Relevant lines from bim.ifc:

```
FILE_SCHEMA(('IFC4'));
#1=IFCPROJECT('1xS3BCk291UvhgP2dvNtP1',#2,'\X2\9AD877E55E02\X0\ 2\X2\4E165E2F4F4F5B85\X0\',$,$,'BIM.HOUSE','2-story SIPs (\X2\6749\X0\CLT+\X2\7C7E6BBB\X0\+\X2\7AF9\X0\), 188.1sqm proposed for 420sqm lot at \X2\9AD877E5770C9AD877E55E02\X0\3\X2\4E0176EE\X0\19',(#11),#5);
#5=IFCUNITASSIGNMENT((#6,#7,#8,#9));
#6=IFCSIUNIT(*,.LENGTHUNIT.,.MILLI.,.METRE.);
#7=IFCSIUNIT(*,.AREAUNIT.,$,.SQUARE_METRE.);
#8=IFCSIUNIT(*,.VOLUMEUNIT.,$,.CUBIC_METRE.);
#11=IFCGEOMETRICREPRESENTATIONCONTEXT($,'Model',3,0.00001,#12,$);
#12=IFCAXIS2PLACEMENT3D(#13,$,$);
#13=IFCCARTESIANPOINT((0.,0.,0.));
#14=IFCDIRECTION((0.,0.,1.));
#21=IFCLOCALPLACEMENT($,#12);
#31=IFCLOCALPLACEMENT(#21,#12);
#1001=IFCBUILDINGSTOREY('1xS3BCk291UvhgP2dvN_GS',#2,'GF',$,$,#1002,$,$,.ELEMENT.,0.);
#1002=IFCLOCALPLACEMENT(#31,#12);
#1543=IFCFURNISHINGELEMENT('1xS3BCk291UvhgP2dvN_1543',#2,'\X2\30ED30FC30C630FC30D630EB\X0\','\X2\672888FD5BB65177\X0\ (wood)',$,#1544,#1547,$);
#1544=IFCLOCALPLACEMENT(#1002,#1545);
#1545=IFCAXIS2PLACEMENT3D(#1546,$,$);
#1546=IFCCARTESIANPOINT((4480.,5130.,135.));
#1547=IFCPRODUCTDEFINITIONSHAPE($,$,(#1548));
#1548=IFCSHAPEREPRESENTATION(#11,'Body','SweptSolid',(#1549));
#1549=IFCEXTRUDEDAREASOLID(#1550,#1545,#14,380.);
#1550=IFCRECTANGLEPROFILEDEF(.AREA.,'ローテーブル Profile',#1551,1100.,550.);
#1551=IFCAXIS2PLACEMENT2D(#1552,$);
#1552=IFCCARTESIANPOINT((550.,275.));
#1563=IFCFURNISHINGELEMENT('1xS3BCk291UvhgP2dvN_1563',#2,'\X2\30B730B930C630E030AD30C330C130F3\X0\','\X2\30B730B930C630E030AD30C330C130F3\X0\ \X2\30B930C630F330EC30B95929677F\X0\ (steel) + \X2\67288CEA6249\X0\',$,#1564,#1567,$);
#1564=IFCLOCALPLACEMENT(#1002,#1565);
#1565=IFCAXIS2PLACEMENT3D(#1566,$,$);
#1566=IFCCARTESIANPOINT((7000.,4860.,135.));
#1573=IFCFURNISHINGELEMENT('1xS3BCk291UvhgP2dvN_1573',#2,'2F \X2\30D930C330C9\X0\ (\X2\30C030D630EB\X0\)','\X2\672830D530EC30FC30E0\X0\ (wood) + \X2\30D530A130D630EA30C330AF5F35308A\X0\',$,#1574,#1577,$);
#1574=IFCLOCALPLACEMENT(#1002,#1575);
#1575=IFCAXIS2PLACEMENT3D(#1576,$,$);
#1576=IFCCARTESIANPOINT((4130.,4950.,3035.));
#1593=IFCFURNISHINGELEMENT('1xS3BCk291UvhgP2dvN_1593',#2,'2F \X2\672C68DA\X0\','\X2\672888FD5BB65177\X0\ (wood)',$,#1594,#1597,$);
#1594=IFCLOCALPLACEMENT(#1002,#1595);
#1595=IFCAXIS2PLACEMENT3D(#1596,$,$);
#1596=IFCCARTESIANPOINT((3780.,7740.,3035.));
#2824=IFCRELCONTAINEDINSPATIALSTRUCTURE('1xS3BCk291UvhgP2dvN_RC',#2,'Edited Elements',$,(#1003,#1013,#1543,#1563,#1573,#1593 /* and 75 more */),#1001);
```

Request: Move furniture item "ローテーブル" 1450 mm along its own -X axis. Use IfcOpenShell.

```python
import ifcopenshell
import ifcopenshell.api.geometry
import ifcopenshell.util.placement
import ifcopenshell.util.unit

model = ifcopenshell.open("bim.ifc")
unit_scale = ifcopenshell.util.unit.calculate_unit_scale(model)

item = model.by_id(1543)
matrix = ifcopenshell.util.placement.get_local_placement(item.ObjectPlacement)
matrix[:3, 3] -= matrix[:3, 0] * 1.45 / unit_scale
ifcopenshell.api.geometry.edit_object_placement(model, product=item, matrix=matrix, is_si=False)

print(ifcopenshell.util.placement.get_local_placement(item.ObjectPlacement).round(3) + 0.0)

model.write("bim-out.ifc")
```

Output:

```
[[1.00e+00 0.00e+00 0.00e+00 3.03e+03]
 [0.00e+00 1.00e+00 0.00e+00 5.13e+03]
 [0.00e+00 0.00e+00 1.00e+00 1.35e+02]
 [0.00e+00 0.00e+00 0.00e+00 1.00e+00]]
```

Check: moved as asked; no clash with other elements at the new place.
